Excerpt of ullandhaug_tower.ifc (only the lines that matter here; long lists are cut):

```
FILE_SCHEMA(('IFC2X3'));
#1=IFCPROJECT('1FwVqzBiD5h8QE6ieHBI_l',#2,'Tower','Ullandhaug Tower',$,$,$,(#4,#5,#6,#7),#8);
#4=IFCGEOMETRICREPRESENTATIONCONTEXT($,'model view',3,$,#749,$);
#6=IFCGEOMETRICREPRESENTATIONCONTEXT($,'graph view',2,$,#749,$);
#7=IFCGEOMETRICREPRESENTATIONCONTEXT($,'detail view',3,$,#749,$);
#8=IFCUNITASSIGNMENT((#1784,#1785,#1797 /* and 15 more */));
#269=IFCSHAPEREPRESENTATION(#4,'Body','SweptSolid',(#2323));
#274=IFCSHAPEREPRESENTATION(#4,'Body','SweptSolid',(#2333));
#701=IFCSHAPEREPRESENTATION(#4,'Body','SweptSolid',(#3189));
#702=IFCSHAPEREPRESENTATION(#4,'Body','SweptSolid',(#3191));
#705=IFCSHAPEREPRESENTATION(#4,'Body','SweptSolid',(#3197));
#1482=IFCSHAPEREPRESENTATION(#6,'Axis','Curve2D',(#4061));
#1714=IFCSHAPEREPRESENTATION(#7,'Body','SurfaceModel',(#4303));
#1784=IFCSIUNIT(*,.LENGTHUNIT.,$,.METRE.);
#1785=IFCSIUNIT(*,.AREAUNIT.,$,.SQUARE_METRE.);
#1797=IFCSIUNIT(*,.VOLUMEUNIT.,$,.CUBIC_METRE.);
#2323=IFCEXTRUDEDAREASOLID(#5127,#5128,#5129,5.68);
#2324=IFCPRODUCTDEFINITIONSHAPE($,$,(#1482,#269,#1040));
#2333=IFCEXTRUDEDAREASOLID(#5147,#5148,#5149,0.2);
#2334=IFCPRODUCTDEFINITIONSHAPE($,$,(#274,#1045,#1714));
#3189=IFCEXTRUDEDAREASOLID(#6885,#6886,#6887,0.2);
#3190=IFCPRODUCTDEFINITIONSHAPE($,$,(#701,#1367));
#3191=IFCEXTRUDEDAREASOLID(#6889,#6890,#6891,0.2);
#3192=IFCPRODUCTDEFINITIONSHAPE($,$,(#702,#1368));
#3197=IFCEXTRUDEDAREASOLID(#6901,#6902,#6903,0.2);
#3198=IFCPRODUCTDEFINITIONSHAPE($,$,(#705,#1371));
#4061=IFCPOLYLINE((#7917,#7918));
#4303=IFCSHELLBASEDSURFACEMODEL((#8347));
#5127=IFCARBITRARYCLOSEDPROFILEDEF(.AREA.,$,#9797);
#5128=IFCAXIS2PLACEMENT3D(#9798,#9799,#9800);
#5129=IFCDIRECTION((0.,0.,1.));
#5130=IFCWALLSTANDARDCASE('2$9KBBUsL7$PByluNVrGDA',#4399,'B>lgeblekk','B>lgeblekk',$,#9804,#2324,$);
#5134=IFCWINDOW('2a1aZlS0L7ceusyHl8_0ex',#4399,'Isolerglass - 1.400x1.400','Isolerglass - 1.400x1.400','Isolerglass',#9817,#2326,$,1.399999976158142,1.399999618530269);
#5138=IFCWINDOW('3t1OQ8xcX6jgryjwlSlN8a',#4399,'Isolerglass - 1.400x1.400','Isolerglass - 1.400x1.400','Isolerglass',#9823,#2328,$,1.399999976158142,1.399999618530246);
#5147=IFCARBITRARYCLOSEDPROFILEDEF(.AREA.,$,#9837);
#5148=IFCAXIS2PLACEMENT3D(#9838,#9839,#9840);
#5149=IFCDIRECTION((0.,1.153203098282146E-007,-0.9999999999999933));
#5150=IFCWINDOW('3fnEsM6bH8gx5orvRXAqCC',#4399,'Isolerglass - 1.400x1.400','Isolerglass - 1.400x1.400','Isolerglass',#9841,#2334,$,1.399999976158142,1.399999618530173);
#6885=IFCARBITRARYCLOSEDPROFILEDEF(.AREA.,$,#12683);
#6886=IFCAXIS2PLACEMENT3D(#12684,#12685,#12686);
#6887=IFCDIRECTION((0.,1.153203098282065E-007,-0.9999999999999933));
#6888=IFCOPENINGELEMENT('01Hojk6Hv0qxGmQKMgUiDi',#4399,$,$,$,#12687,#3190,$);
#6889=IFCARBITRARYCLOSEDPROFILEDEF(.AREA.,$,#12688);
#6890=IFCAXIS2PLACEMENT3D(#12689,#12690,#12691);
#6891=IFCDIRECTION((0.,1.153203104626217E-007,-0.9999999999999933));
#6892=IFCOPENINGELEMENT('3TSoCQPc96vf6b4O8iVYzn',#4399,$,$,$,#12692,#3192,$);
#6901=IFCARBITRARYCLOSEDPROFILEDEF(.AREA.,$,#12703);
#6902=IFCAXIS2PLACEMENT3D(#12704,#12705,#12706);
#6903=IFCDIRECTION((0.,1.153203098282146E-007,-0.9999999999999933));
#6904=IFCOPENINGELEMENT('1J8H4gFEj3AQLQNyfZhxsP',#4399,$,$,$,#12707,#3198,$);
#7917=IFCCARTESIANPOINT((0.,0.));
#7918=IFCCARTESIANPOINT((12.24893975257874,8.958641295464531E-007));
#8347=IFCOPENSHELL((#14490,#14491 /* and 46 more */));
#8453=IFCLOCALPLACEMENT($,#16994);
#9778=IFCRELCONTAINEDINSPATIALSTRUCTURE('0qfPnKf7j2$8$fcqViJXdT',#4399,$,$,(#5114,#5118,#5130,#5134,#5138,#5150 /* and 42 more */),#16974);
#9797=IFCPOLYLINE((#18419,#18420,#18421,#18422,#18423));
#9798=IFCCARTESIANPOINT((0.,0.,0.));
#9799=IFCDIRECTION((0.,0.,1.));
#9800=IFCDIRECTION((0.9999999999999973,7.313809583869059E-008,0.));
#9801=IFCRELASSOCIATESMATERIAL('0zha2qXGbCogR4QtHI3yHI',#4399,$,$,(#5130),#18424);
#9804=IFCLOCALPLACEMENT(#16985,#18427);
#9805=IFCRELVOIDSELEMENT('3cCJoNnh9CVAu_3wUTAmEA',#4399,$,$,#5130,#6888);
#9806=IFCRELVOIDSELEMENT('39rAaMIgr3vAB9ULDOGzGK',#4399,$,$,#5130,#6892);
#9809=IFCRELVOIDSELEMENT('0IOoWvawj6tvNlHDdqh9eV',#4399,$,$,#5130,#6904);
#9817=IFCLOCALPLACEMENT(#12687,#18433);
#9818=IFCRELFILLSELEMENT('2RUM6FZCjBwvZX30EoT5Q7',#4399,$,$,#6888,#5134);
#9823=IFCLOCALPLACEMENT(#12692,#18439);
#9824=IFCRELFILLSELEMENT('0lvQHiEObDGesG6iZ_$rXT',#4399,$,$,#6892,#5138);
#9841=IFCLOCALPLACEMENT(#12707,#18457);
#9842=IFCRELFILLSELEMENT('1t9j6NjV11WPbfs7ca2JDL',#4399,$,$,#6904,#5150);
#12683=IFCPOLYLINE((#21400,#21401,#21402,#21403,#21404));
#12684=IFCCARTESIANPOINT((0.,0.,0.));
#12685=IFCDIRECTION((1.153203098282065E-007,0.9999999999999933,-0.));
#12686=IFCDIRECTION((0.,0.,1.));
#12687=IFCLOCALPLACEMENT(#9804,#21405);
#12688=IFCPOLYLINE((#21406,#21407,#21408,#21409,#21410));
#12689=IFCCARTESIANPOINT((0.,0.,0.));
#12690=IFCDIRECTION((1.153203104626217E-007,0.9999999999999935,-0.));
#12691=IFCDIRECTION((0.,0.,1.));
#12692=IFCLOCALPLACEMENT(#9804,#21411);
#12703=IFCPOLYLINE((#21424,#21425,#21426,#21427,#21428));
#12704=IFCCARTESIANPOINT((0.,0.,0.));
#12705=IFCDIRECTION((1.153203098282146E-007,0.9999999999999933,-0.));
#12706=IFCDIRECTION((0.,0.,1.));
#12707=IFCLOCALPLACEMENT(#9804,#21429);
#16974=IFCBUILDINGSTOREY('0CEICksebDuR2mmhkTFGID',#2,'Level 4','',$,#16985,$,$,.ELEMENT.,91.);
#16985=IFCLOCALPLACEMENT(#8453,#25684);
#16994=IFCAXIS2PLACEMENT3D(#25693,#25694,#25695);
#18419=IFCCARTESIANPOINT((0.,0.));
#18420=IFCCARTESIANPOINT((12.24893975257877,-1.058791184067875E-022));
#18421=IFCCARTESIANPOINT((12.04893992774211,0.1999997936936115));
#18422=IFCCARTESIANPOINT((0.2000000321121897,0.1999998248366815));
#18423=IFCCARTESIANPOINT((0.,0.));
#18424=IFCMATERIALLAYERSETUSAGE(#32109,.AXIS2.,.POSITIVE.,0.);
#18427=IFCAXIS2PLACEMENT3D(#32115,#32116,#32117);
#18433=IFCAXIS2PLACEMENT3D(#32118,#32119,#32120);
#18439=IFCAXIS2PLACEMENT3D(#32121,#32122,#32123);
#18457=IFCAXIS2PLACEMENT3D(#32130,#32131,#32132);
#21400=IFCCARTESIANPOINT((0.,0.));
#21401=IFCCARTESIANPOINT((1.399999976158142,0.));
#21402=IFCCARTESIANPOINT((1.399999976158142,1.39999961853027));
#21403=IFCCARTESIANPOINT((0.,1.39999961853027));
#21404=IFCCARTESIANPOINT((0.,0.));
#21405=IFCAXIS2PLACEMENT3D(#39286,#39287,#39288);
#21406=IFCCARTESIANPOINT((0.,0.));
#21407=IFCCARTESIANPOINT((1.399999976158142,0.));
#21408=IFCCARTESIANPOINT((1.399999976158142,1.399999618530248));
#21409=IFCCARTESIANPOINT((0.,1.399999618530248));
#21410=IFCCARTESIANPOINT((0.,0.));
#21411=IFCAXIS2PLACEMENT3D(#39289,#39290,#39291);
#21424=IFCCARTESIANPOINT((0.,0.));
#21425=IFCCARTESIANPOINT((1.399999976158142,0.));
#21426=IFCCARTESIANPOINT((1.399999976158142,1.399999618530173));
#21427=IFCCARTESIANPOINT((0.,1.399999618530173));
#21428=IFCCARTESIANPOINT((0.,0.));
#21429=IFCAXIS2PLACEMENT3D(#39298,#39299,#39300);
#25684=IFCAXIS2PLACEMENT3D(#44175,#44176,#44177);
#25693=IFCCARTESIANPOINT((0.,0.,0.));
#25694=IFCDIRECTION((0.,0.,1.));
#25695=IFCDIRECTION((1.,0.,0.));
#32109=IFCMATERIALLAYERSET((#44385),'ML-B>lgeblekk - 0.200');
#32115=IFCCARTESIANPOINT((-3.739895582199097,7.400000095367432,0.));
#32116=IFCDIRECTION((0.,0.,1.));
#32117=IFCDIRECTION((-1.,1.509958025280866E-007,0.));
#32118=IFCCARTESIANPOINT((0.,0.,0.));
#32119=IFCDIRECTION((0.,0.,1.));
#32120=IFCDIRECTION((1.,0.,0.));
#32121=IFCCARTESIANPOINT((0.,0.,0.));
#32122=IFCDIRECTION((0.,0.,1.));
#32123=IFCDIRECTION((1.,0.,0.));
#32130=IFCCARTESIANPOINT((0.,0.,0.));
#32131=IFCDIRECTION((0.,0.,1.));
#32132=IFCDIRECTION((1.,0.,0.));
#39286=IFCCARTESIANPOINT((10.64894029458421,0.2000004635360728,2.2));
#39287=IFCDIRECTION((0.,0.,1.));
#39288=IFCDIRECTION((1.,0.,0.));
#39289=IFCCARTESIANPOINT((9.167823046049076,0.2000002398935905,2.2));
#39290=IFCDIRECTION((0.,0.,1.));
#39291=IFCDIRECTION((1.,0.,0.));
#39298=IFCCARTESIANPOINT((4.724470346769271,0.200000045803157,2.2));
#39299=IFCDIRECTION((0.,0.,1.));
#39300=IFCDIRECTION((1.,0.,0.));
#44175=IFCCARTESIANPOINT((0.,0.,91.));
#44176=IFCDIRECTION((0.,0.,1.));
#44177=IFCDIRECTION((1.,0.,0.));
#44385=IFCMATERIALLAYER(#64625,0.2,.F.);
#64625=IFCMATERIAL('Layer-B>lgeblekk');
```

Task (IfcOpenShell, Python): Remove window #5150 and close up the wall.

```python
import ifcopenshell
import ifcopenshell.api.feature
import ifcopenshell.api.root
import ifcopenshell.geom
import ifcopenshell.util.shape

model = ifcopenshell.open("ullandhaug_tower.ifc")
settings = ifcopenshell.geom.settings()


def volume(element):
    """Net volume in cubic metres, openings subtracted."""
    shape = ifcopenshell.geom.create_shape(settings, element)
    return ifcopenshell.util.shape.get_volume(shape.geometry)


window = model.by_guid("3fnEsM6bH8gx5orvRXAqCC")
opening = window.FillsVoids[0].RelatingOpeningElement
wall = opening.VoidsElements[0].RelatingBuildingElement
before = volume(wall)

ifcopenshell.api.root.remove_product(model, product=window)
ifcopenshell.api.feature.remove_feature(model, feature=opening)

after = volume(wall)

print(f"wall volume {before:.3f} -> {after:.3f} m3")

model.write("ullandhaug_tower_edited.ifc")
```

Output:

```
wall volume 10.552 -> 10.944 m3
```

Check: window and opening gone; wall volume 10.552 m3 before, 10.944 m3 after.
